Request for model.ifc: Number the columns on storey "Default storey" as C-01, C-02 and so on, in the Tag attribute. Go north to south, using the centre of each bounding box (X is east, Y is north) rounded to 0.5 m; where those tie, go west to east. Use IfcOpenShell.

First a look at what the model holds.

```python
import ifcopenshell
import ifcopenshell.util.element
import ifcopenshell.util.placement

model = ifcopenshell.open("model.ifc")
print(model.schema)
storey = next(s for s in model.by_type("IfcBuildingStorey") if s.Name == "Default storey")
columns = [e for e in ifcopenshell.util.element.get_decomposition(storey) if e.is_a("IfcColumn")]
for e in sorted(columns, key=lambda e: e.id()):
    origin = ifcopenshell.util.placement.get_local_placement(e.ObjectPlacement)[:3, 3]
    print(e.id(), e.Tag, e.Name, origin.round(2) + 0.0, sep=" | ")
```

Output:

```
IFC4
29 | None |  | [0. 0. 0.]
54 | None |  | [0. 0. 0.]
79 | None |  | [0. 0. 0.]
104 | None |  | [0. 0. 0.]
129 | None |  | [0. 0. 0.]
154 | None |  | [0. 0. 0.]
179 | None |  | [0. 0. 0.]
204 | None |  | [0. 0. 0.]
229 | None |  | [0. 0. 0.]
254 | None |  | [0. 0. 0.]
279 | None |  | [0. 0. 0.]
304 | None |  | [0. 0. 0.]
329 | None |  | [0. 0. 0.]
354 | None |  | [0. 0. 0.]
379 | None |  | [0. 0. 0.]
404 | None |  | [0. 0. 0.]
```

```python
import ifcopenshell
import ifcopenshell.geom
import ifcopenshell.util.element
import ifcopenshell.util.shape

model = ifcopenshell.open("model.ifc")
settings = ifcopenshell.geom.settings()
settings.set("use-world-coords", True)


def centre(element):
    shape = ifcopenshell.geom.create_shape(settings, element)
    return ifcopenshell.util.shape.get_bbox_centroid(shape.geometry)


storey = next(s for s in model.by_type("IfcBuildingStorey") if s.Name == "Default storey")
columns = [e for e in ifcopenshell.util.element.get_decomposition(storey) if e.is_a("IfcColumn")]

# Insertion points can sit at a corner or the storey origin, so sort by the geometry (in metres).
centres = {e: centre(e) for e in columns}
columns.sort(key=lambda e: (-round(centres[e][1] / 0.5), centres[e][0]))

for i, e in enumerate(columns, start=1):
    number = f"C-{i:02d}"
    e.Tag = number
    print(e.id(), number)

model.write("model_edited.ifc")
```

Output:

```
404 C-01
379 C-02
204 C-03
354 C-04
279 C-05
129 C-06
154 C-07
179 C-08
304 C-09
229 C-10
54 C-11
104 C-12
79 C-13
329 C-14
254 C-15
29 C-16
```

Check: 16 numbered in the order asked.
